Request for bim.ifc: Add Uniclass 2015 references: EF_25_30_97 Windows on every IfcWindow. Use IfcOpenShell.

First a look at what the model holds.

```python
import ifcopenshell

model = ifcopenshell.open("bim.ifc")
print(model.schema)
print("classifications:", [c.Name for c in model.by_type("IfcClassification")])
for ifc_class in ("IfcDoor", "IfcRoof", "IfcStair", "IfcWall", "IfcWindow"):
    print(ifc_class, len(model.by_type(ifc_class)))
```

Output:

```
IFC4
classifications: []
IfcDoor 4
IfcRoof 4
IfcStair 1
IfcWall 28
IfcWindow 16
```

```python
import ifcopenshell
import ifcopenshell.api.classification

model = ifcopenshell.open("bim.ifc")

system = ifcopenshell.api.classification.add_classification(model, classification="Uniclass 2015")

codes = {
    "IfcWindow": ("EF_25_30_97", "Windows"),
}
for ifc_class, (code, name) in codes.items():
    products = model.by_type(ifc_class)
    ifcopenshell.api.classification.add_reference(
        model, products=products, classification=system, identification=code, name=name
    )
    print(code, len(products))

model.write("bim_updated.ifc")
```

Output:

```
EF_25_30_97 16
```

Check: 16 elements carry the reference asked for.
